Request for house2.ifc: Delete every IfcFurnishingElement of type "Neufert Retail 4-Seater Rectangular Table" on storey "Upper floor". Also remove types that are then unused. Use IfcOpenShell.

First a look at what the model holds.

```python
import ifcopenshell
import ifcopenshell.util.element

model = ifcopenshell.open("house2.ifc")
print(model.schema)
storey = next(s for s in model.by_type("IfcBuildingStorey") if s.Name == "Upper floor")
furniture = [e for e in ifcopenshell.util.element.get_decomposition(storey) if e.is_a("IfcFurnishingElement")]
seen = {}
for e in furniture:
    element_type = ifcopenshell.util.element.get_type(e)
    name = element_type.Name if element_type not in (None, e) else None
    seen[name] = seen.get(name, 0) + 1
for name, count in sorted(seen.items(), key=str):
    print(count, "x", name)
```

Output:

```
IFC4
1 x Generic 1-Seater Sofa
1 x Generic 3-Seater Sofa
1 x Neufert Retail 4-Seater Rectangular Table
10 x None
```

```python
import ifcopenshell
import ifcopenshell.api.root
import ifcopenshell.util.element

model = ifcopenshell.open("house2.ifc")

storey = next(s for s in model.by_type("IfcBuildingStorey") if s.Name == "Upper floor")
furniture = [e for e in ifcopenshell.util.element.get_decomposition(storey) if e.is_a("IfcFurnishingElement")]
targets = [e for e in furniture if (t := ifcopenshell.util.element.get_type(e)) not in (None, e) and t.Name == "Neufert Retail 4-Seater Rectangular Table"]
types = {ifcopenshell.util.element.get_type(e) for e in targets} - {None, *targets}

for e in targets:
    ifcopenshell.api.root.remove_product(model, product=e)
print(len(targets), "removed")

unused = [t for t in types if not ifcopenshell.util.element.get_types(t)]
for t in unused:
    ifcopenshell.api.root.remove_product(model, product=t)
print(len(unused), "unused types removed")

model.write("house2_v2.ifc")
```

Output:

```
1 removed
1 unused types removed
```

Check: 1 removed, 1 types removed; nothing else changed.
